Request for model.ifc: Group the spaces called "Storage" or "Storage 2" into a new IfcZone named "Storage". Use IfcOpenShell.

First a look at what the model holds.

```python
import ifcopenshell

model = ifcopenshell.open("model.ifc")
print(model.schema)
seen = {}
for space in model.by_type("IfcSpace"):
    seen[space.LongName] = seen.get(space.LongName, 0) + 1
for name, count in sorted(seen.items(), key=str):
    print(count, "x", name)
print("zones:", [z.Name for z in model.by_type("IfcZone")][:20])
```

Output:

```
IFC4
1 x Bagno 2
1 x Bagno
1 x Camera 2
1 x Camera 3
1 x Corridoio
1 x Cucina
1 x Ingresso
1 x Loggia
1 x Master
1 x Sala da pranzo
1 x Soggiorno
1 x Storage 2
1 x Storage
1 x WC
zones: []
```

```python
import ifcopenshell
import ifcopenshell.api.group
import ifcopenshell.api.root

model = ifcopenshell.open("model.ifc")

names = {"Storage", "Storage 2"}
spaces = [s for s in model.by_type("IfcSpace") if s.LongName in names]

zone = ifcopenshell.api.root.create_entity(model, ifc_class="IfcZone", name="Storage")
ifcopenshell.api.group.assign_group(model, products=spaces, group=zone)
print(len(spaces), "spaces in", zone.Name)

model.write("model_edited.ifc")
```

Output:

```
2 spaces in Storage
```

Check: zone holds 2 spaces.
